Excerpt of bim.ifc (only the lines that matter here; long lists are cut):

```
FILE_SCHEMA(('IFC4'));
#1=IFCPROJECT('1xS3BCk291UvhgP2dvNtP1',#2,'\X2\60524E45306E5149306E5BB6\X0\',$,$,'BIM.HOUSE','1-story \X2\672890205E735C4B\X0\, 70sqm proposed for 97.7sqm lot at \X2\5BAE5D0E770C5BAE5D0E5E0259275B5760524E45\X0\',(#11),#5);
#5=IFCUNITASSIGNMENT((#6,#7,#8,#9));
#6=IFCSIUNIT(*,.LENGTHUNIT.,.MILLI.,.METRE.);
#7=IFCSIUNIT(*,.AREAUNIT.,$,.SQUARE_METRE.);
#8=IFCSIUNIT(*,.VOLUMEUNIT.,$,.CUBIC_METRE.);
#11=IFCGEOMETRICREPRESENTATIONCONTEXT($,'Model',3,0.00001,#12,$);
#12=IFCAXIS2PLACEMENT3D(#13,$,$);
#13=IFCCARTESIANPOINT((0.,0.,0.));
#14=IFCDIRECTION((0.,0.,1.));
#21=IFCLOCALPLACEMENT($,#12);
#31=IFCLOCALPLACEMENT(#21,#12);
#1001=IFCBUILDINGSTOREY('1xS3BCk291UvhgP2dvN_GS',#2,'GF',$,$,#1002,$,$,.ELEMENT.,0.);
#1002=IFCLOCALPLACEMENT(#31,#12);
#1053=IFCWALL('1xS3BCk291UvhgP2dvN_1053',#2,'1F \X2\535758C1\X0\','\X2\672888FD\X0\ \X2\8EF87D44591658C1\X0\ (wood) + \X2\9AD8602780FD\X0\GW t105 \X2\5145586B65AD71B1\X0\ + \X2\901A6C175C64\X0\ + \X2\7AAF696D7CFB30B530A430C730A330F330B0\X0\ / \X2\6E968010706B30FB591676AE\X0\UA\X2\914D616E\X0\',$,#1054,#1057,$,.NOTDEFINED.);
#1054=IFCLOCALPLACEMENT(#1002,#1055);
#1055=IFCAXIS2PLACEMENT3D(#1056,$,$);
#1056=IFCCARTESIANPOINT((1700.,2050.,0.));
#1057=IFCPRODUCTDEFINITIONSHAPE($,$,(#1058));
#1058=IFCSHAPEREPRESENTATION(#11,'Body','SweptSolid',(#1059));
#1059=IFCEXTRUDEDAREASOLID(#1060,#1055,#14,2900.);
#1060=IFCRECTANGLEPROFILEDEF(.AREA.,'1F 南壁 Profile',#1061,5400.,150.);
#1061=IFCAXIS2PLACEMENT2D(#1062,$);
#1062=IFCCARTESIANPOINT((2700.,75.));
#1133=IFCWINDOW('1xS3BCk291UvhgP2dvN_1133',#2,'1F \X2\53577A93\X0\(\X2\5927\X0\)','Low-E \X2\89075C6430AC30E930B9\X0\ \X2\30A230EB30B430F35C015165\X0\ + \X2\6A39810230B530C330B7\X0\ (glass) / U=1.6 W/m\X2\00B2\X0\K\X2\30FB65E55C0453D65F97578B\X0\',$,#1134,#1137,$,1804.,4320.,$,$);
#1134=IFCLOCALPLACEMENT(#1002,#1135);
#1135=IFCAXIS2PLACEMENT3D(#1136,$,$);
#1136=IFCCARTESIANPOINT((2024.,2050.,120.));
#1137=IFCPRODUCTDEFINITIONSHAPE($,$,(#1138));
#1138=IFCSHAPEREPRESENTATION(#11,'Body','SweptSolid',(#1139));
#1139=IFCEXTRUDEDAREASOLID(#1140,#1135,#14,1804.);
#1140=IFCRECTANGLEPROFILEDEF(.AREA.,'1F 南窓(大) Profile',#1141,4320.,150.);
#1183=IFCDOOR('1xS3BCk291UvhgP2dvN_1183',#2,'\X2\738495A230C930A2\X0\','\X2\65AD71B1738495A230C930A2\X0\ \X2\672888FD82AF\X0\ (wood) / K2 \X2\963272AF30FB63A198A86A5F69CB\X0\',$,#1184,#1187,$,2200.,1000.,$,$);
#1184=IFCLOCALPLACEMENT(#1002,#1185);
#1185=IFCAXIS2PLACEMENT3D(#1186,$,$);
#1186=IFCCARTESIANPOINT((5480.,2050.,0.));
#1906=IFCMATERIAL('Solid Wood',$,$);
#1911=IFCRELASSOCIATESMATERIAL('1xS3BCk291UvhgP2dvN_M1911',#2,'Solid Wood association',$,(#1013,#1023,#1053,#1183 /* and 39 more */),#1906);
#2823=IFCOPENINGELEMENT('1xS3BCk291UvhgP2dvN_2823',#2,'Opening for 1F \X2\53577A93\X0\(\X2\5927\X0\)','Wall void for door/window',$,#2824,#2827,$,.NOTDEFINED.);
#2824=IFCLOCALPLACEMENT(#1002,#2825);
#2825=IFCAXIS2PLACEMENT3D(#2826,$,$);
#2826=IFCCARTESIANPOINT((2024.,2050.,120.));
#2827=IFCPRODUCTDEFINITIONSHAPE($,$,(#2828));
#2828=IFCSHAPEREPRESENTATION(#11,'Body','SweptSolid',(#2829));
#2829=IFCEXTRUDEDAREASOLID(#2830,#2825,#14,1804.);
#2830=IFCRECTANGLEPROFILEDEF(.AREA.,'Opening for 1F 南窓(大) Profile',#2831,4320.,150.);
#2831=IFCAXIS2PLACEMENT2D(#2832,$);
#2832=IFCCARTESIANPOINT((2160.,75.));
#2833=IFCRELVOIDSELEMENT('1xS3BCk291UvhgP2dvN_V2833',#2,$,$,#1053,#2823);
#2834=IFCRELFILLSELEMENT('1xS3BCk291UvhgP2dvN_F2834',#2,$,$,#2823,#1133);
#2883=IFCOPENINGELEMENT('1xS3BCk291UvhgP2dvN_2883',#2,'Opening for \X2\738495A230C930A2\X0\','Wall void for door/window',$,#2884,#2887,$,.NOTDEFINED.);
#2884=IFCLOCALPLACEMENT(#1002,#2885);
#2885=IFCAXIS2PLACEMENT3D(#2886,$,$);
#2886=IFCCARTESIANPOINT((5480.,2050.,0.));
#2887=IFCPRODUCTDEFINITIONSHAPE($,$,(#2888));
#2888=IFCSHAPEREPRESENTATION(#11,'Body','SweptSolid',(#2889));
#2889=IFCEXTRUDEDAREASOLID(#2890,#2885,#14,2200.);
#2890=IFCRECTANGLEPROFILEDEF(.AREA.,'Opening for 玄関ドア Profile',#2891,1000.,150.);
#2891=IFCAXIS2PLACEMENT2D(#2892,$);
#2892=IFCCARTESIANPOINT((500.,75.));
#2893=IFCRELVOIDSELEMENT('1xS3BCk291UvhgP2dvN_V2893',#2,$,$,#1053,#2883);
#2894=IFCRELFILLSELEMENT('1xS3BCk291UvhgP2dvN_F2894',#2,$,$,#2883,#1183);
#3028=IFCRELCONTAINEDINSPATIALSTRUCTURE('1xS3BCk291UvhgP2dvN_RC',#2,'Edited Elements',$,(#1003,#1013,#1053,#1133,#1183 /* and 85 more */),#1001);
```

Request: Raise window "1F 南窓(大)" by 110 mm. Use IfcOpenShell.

```python
import numpy as np
import ifcopenshell
import ifcopenshell.api.geometry
import ifcopenshell.util.placement
import ifcopenshell.util.unit

model = ifcopenshell.open("bim.ifc")
unit_scale = ifcopenshell.util.unit.calculate_unit_scale(model)

window = model.by_guid("1xS3BCk291UvhgP2dvN_1133")
opening = window.FillsVoids[0].RelatingOpeningElement
dz = 0.11 / unit_scale

shift = np.array([0.0, 0.0, dz])
# The window is not placed relative to its opening, so move both.
for product in (opening, window):
    matrix = ifcopenshell.util.placement.get_local_placement(product.ObjectPlacement)
    matrix[:3, 3] += shift
    ifcopenshell.api.geometry.edit_object_placement(model, product=product, matrix=matrix, is_si=False)

print(f"moved by {dz * unit_scale:+.3f} m")

model.write("bim_edited.ifc")
```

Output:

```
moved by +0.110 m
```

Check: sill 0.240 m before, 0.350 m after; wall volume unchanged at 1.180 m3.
